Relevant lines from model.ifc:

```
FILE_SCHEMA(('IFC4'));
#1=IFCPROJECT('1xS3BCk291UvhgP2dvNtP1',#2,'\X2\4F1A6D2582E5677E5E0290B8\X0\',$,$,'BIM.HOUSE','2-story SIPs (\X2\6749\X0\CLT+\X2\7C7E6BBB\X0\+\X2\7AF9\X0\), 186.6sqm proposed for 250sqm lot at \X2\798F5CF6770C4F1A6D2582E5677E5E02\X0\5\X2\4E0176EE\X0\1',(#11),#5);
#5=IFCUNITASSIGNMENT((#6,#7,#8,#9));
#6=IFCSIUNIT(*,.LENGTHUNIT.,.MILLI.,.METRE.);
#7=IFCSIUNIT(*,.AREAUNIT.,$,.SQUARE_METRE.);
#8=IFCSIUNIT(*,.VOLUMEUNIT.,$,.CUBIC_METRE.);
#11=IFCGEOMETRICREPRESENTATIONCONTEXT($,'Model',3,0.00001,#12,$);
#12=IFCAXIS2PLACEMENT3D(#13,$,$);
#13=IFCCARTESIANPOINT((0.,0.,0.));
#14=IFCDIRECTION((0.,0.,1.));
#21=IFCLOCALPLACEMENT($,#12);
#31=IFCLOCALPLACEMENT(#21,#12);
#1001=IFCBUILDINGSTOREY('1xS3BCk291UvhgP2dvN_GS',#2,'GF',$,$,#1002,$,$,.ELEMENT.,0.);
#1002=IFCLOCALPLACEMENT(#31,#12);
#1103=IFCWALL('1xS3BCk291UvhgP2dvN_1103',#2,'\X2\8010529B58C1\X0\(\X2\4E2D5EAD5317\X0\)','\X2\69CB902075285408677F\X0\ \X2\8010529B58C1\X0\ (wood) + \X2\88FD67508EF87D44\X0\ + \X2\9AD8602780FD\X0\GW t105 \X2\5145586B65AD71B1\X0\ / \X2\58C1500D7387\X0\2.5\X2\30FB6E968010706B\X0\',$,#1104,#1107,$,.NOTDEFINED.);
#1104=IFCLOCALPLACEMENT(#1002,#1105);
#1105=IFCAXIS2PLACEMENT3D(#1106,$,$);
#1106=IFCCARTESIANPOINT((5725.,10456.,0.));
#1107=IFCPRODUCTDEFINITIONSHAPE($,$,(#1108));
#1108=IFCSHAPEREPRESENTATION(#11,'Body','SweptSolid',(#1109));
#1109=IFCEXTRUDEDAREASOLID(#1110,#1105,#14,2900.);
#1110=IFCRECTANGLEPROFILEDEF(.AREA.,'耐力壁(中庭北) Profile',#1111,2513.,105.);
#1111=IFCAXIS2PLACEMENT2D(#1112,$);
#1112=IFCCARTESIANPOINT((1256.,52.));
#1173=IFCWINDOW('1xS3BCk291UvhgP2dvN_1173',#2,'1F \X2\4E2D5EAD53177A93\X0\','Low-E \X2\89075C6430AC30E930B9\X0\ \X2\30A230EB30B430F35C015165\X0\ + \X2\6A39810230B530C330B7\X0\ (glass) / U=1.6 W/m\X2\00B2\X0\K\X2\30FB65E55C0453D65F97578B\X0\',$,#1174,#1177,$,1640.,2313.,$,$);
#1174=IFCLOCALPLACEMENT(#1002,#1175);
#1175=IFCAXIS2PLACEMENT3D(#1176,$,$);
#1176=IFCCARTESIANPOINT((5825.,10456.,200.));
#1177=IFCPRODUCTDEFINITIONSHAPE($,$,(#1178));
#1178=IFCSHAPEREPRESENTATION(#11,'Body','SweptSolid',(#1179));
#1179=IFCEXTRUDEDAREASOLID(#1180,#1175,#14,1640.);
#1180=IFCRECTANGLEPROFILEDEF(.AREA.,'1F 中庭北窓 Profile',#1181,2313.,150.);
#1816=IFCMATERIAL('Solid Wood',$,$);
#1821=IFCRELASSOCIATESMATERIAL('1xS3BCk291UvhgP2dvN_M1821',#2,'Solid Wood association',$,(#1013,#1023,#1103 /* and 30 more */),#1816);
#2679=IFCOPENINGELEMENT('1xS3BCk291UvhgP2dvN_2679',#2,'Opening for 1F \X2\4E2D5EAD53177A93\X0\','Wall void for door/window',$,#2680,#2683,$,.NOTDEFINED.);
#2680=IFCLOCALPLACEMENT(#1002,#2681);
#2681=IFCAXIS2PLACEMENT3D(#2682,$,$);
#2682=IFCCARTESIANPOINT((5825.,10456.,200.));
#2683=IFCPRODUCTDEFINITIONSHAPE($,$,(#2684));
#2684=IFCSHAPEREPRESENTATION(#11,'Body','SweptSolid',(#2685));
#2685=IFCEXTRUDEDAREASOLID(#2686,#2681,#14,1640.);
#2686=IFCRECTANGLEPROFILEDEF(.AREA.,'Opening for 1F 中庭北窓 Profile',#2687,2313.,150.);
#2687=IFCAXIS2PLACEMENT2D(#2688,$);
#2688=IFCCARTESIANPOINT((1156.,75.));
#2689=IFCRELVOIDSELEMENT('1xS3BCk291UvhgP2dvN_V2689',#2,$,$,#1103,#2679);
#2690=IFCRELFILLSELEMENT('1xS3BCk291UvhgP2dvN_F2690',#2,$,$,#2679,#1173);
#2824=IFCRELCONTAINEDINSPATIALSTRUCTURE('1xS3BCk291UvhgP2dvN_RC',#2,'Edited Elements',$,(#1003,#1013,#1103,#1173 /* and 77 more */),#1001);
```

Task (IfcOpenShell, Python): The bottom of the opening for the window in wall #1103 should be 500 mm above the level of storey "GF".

```python
import numpy as np
import ifcopenshell
import ifcopenshell.api.geometry
import ifcopenshell.geom
import ifcopenshell.util.element
import ifcopenshell.util.placement
import ifcopenshell.util.shape
import ifcopenshell.util.unit

model = ifcopenshell.open("model.ifc")
unit_scale = ifcopenshell.util.unit.calculate_unit_scale(model)

window = model.by_guid("1xS3BCk291UvhgP2dvN_1173")
opening = window.FillsVoids[0].RelatingOpeningElement
storey = ifcopenshell.util.element.get_container(window, ifc_class="IfcBuildingStorey")
level = ifcopenshell.util.placement.get_local_placement(storey.ObjectPlacement)[2, 3]

# The opening's origin need not be at the sill, so measure its lowest point.
shape = ifcopenshell.geom.create_shape(ifcopenshell.geom.settings(), opening)
bottom = ifcopenshell.util.shape.get_shape_bottom_elevation(shape, shape.geometry) / unit_scale
dz = level + 500.0 - bottom

shift = np.array([0.0, 0.0, dz])
# The window is not placed relative to its opening, so move both.
for product in (opening, window):
    matrix = ifcopenshell.util.placement.get_local_placement(product.ObjectPlacement)
    matrix[:3, 3] += shift
    ifcopenshell.api.geometry.edit_object_placement(model, product=product, matrix=matrix, is_si=False)

print(f"moved by {dz * unit_scale:+.3f} m")

model.write("model_updated.ifc")
```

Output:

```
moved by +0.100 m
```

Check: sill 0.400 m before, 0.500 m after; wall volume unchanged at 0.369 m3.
